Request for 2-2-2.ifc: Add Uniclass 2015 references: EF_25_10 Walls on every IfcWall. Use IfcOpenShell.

First a look at what the model holds.

```python
import ifcopenshell

model = ifcopenshell.open("2-2-2.ifc")
print(model.schema)
print("classifications:", [c.Name for c in model.by_type("IfcClassification")])
for ifc_class in ("IfcDoor", "IfcRoof", "IfcStair", "IfcWall", "IfcWindow"):
    print(ifc_class, len(model.by_type(ifc_class)))
```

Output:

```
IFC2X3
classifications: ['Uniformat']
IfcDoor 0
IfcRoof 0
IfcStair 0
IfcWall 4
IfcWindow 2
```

```python
import ifcopenshell
import ifcopenshell.api.classification

model = ifcopenshell.open("2-2-2.ifc")

# IFC2X3 requires Source and Edition and has no link from the project to the system.
system = model.create_entity("IfcClassification", Source="NBS", Edition="2015", Name="Uniclass 2015")

codes = {
    "IfcWall": ("EF_25_10", "Walls"),
}
for ifc_class, (code, name) in codes.items():
    products = model.by_type(ifc_class)
    ifcopenshell.api.classification.add_reference(
        model, products=products, classification=system, identification=code, name=name
    )
    print(code, len(products))

model.write("2-2-2_updated.ifc")
```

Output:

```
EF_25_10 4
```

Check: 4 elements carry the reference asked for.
